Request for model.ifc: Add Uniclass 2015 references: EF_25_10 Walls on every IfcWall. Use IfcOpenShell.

First a look at what the model holds.

```python
import ifcopenshell

model = ifcopenshell.open("model.ifc")
print(model.schema)
print("classifications:", [c.Name for c in model.by_type("IfcClassification")])
for ifc_class in ("IfcDoor", "IfcRoof", "IfcStair", "IfcWall", "IfcWindow"):
    print(ifc_class, len(model.by_type(ifc_class)))
```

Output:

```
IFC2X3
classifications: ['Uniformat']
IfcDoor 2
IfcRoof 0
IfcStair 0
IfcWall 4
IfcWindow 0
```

```python
import ifcopenshell
import ifcopenshell.api.classification

model = ifcopenshell.open("model.ifc")

# IFC2X3 requires Source and Edition and has no link from the project to the system.
system = model.create_entity("IfcClassification", Source="NBS", Edition="2015", Name="Uniclass 2015")

codes = {
    "IfcWall": ("EF_25_10", "Walls"),
}
for ifc_class, (code, name) in codes.items():
    products = model.by_type(ifc_class)
    ifcopenshell.api.classification.add_reference(
        model, products=products, classification=system, identification=code, name=name
    )
    print(code, len(products))

model.write("model_edited.ifc")
```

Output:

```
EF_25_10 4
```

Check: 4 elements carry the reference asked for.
